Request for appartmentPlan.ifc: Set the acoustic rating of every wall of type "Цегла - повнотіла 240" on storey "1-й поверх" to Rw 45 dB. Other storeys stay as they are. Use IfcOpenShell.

First a look at what the model holds.

```python
import ifcopenshell
import ifcopenshell.util.element

model = ifcopenshell.open("appartmentPlan.ifc")
print(model.schema)
storey = next(s for s in model.by_type("IfcBuildingStorey") if s.Name == "1-й поверх")
walls = [e for e in ifcopenshell.util.element.get_decomposition(storey) if e.is_a("IfcWall")]
seen = {}
for e in walls:
    element_type = ifcopenshell.util.element.get_type(e)
    key = (element_type.Name if element_type != e and element_type else None, ifcopenshell.util.element.get_pset(e, "Pset_WallCommon", "AcousticRating"))
    seen[key] = seen.get(key, 0) + 1
for (name, value), count in sorted(seen.items(), key=str):
    print(count, "x", name, "|", value)
```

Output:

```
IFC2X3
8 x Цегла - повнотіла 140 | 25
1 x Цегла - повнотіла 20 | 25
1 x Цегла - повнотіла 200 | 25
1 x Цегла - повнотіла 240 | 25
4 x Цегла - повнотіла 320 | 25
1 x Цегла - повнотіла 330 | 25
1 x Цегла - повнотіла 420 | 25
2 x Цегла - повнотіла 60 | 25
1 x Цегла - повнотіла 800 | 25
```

```python
import ifcopenshell
import ifcopenshell.api.pset
import ifcopenshell.util.element

model = ifcopenshell.open("appartmentPlan.ifc")

storey = next(s for s in model.by_type("IfcBuildingStorey") if s.Name == "1-й поверх")
walls = [e for e in ifcopenshell.util.element.get_decomposition(storey) if e.is_a("IfcWall")]

count = 0
for e in walls:
    element_type = ifcopenshell.util.element.get_type(e)
    if element_type in (None, e) or element_type.Name != "Цегла - повнотіла 240":
        continue
    # add_pset returns the element's existing set when there is one.
    pset = ifcopenshell.api.pset.add_pset(model, product=e, name="Pset_WallCommon")
    ifcopenshell.api.pset.edit_pset(model, pset=pset, properties={"AcousticRating": "Rw 45 dB"})
    count += 1

print(count, "walls updated")

model.write("appartmentPlan_edited.ifc")
```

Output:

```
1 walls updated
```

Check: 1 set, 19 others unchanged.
